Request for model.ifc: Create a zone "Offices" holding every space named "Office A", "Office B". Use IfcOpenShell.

First a look at what the model holds.

```python
import ifcopenshell

model = ifcopenshell.open("model.ifc")
print(model.schema)
seen = {}
for space in model.by_type("IfcSpace"):
    seen[space.Name] = seen.get(space.Name, 0) + 1
for name, count in sorted(seen.items(), key=str):
    print(count, "x", name)
print("zones:", [z.Name for z in model.by_type("IfcZone")][:20])
```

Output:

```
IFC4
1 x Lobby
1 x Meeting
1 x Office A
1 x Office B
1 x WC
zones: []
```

```python
import ifcopenshell
import ifcopenshell.api.group
import ifcopenshell.api.root

model = ifcopenshell.open("model.ifc")

names = {"Office A", "Office B"}
spaces = [s for s in model.by_type("IfcSpace") if s.Name in names]

zone = ifcopenshell.api.root.create_entity(model, ifc_class="IfcZone", name="Offices")
ifcopenshell.api.group.assign_group(model, products=spaces, group=zone)
print(len(spaces), "spaces in", zone.Name)

model.write("model_rev.ifc")
```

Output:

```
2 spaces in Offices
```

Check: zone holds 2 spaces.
